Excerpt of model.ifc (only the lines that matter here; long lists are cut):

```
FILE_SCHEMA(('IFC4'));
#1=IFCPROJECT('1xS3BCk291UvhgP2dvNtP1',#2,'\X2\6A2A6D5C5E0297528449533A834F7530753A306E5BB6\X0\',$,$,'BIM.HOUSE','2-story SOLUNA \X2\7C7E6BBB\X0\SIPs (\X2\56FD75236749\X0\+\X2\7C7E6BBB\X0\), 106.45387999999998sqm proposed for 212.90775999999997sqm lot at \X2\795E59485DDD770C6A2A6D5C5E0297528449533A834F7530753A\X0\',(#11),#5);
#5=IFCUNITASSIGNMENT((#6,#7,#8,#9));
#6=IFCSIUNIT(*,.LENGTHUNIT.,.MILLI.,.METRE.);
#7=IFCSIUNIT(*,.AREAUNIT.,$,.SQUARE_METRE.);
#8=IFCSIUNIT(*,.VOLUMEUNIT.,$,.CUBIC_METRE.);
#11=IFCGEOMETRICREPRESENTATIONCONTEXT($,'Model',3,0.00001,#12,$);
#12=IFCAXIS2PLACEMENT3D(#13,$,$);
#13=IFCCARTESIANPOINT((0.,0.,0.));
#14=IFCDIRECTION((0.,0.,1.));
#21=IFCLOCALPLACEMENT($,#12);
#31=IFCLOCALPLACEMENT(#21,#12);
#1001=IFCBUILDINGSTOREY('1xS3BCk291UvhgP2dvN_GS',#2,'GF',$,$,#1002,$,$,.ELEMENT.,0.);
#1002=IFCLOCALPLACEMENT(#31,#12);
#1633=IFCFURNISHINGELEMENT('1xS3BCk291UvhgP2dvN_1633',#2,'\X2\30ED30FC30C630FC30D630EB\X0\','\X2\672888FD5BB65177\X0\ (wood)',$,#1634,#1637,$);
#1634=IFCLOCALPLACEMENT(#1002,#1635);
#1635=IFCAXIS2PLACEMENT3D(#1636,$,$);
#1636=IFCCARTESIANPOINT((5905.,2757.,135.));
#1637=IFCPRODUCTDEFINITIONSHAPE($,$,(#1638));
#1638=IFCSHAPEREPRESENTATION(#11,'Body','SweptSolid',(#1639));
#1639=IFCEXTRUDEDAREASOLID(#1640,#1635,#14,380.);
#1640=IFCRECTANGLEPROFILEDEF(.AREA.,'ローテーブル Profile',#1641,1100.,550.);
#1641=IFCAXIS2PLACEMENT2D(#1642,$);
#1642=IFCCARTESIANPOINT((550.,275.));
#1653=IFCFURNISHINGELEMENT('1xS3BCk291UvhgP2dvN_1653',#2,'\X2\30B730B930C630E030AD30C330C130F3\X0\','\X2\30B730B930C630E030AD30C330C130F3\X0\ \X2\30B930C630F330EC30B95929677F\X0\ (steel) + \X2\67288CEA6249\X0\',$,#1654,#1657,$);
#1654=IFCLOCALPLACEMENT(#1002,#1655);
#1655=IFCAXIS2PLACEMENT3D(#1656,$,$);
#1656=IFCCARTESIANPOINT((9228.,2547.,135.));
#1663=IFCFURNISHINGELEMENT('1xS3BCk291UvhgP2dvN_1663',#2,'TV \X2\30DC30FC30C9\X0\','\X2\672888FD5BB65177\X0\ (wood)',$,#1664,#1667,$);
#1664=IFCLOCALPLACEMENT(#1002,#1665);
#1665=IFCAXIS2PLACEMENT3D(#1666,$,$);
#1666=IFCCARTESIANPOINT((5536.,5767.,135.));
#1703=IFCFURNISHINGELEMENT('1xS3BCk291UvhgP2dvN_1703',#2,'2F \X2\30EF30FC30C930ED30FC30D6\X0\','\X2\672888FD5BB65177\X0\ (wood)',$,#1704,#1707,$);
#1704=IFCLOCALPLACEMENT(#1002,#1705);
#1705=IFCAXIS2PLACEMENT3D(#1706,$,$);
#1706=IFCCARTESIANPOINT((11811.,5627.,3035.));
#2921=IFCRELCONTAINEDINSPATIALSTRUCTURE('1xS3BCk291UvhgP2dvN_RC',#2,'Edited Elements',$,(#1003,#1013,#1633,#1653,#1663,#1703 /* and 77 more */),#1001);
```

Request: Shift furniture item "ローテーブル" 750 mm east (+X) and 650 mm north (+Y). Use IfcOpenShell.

```python
import ifcopenshell
import ifcopenshell.api.geometry
import ifcopenshell.util.placement

model = ifcopenshell.open("model.ifc")

item = model.by_guid("1xS3BCk291UvhgP2dvN_1633")
matrix = ifcopenshell.util.placement.get_local_placement(item.ObjectPlacement)
matrix[0, 3] += 750.0
matrix[1, 3] += 650.0
ifcopenshell.api.geometry.edit_object_placement(model, product=item, matrix=matrix, is_si=False)

print(ifcopenshell.util.placement.get_local_placement(item.ObjectPlacement).round(3) + 0.0)

model.write("model-out.ifc")
```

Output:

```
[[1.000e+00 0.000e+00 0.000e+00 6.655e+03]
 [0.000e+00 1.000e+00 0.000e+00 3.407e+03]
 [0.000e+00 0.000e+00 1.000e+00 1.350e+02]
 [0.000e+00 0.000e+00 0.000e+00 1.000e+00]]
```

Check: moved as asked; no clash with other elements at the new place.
